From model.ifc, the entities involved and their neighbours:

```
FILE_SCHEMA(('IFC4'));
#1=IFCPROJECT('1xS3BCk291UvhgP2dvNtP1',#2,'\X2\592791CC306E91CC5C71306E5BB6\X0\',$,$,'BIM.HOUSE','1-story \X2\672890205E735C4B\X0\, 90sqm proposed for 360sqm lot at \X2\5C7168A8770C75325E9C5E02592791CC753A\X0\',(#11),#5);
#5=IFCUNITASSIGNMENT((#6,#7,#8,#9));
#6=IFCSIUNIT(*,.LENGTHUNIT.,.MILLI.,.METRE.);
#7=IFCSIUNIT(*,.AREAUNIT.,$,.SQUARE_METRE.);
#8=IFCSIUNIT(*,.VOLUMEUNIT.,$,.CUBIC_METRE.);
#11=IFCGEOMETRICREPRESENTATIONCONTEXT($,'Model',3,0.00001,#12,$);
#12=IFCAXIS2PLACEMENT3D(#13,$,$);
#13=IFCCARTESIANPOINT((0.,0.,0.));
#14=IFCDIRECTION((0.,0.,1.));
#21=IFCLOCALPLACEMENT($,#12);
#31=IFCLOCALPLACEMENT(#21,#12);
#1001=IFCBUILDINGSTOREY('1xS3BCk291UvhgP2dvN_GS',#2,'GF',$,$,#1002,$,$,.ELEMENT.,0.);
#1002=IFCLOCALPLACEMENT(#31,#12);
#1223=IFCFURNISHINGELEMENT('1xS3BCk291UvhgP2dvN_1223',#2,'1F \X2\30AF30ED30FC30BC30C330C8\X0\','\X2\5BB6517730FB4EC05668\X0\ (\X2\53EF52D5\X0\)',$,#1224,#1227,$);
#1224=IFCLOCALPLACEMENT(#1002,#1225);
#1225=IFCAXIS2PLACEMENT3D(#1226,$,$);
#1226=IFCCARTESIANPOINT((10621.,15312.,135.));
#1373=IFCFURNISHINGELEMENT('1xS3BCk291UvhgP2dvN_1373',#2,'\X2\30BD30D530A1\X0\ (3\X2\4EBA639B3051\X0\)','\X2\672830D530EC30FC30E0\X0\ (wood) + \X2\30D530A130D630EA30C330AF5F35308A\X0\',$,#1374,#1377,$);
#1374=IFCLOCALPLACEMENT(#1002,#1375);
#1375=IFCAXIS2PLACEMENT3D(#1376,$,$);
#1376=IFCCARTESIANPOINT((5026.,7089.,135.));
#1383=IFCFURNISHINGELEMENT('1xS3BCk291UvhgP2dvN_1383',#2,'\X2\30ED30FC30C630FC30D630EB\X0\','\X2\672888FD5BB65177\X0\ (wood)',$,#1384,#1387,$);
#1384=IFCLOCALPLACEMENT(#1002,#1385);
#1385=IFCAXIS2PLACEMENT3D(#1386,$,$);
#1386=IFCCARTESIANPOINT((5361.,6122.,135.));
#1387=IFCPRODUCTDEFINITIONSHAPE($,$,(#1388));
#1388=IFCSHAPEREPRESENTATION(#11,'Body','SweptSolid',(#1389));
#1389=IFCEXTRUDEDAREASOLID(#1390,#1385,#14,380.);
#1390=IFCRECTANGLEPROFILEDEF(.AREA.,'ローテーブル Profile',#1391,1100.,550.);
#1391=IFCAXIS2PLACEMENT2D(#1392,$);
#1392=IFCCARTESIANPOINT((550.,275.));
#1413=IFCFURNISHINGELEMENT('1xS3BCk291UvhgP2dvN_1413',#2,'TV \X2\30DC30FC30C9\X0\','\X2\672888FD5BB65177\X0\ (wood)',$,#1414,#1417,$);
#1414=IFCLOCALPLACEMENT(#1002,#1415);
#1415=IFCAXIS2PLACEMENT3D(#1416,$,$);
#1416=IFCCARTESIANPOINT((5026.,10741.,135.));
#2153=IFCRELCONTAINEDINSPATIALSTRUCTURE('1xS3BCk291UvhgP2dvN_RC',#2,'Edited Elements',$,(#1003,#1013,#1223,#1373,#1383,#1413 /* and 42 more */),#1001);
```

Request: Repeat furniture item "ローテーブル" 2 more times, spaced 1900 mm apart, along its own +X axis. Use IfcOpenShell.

```python
import ifcopenshell
import ifcopenshell.api.geometry
import ifcopenshell.api.root
import ifcopenshell.util.element
import ifcopenshell.util.placement
import ifcopenshell.util.unit

model = ifcopenshell.open("model.ifc")
unit_scale = ifcopenshell.util.unit.calculate_unit_scale(model)


def reuse_history(source, copy):
    """copy_class also copies each property set's owner history, people and application; keep the originals."""
    for rel in copy.IsDefinedBy:
        if rel.is_a("IfcRelDefinesByProperties") and (history := rel.RelatingPropertyDefinition.OwnerHistory):
            rel.RelatingPropertyDefinition.OwnerHistory = source.OwnerHistory
            ifcopenshell.util.element.remove_deep2(model, history)


source = model.by_guid("1xS3BCk291UvhgP2dvN_1383")
base = ifcopenshell.util.placement.get_local_placement(source.ObjectPlacement)
step = base[:3, 0] * 1.9 / unit_scale

for i in range(1, 3):
    copy = ifcopenshell.api.root.copy_class(model, product=source)
    copy.Representation = ifcopenshell.util.element.copy_deep(
        model, source.Representation, exclude=["IfcGeometricRepresentationContext", "IfcRepresentationMap"]
    )
    reuse_history(source, copy)
    matrix = base.copy()
    matrix[:3, 3] += i * step
    print("added at", matrix[:3, 3].round(3) + 0.0)
    ifcopenshell.api.geometry.edit_object_placement(model, product=copy, matrix=matrix, is_si=False)

model.write("model_edited.ifc")
```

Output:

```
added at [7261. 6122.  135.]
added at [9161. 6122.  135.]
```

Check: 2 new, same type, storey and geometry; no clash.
